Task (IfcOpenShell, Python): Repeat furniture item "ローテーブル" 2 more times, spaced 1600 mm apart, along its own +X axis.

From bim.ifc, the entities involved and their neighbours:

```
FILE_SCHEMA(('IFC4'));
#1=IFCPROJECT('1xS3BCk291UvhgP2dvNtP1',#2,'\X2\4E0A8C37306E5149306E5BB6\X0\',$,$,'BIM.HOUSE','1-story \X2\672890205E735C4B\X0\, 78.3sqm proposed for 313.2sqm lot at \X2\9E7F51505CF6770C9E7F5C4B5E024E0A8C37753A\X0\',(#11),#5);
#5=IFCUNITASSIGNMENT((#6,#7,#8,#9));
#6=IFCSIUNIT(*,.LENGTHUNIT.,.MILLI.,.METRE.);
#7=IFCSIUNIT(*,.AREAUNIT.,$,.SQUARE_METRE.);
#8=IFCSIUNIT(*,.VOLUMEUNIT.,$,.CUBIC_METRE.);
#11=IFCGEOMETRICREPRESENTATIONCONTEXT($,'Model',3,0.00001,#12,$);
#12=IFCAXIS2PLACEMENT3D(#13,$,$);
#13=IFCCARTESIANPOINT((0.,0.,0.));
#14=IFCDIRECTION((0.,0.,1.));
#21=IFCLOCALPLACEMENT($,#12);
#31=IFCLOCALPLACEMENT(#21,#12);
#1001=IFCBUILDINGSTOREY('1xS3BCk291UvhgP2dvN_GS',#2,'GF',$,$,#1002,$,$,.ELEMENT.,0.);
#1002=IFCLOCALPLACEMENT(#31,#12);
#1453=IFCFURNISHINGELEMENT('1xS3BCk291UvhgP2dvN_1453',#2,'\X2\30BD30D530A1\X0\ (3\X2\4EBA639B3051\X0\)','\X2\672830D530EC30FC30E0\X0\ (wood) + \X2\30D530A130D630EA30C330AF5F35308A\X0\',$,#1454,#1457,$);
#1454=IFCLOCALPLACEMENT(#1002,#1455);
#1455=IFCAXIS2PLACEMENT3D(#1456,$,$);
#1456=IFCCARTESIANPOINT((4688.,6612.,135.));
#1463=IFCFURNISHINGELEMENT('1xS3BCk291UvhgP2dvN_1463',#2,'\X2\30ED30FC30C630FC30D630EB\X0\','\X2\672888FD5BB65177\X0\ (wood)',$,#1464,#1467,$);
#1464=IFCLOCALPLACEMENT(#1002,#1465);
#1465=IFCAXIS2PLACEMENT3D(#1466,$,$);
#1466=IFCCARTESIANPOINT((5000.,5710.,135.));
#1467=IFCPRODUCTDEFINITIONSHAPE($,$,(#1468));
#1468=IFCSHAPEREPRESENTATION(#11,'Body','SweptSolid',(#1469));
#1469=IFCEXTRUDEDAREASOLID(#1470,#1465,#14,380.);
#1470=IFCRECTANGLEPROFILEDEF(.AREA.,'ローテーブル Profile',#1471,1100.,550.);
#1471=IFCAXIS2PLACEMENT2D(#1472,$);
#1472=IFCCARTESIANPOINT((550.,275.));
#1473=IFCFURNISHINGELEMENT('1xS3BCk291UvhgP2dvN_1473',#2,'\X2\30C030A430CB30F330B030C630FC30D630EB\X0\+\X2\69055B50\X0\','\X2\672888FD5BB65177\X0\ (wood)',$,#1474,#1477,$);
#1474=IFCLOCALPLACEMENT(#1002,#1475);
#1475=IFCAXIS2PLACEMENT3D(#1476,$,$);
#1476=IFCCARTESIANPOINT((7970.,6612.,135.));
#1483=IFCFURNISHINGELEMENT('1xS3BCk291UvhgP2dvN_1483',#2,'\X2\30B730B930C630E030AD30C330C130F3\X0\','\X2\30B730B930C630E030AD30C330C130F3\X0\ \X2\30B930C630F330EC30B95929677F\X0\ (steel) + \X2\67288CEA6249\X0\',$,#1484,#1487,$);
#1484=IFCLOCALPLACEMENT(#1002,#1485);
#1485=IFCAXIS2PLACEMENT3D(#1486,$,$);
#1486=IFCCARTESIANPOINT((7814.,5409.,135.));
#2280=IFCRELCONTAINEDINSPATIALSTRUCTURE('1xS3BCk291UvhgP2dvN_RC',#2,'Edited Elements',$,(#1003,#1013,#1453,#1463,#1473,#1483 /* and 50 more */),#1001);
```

```python
import ifcopenshell
import ifcopenshell.api.geometry
import ifcopenshell.api.root
import ifcopenshell.util.element
import ifcopenshell.util.placement

model = ifcopenshell.open("bim.ifc")


def reuse_history(source, copy):
    """copy_class also copies each property set's owner history, people and application; keep the originals."""
    for rel in copy.IsDefinedBy:
        if rel.is_a("IfcRelDefinesByProperties") and (history := rel.RelatingPropertyDefinition.OwnerHistory):
            rel.RelatingPropertyDefinition.OwnerHistory = source.OwnerHistory
            ifcopenshell.util.element.remove_deep2(model, history)


source = model.by_guid("1xS3BCk291UvhgP2dvN_1463")
base = ifcopenshell.util.placement.get_local_placement(source.ObjectPlacement)
step = base[:3, 0] * 1600.0

for i in range(1, 3):
    copy = ifcopenshell.api.root.copy_class(model, product=source)
    copy.Representation = ifcopenshell.util.element.copy_deep(
        model, source.Representation, exclude=["IfcGeometricRepresentationContext", "IfcRepresentationMap"]
    )
    reuse_history(source, copy)
    matrix = base.copy()
    matrix[:3, 3] += i * step
    print("added at", matrix[:3, 3].round(3) + 0.0)
    ifcopenshell.api.geometry.edit_object_placement(model, product=copy, matrix=matrix, is_si=False)

model.write("bim_updated.ifc")
```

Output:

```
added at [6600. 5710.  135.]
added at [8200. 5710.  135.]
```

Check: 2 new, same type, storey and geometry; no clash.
